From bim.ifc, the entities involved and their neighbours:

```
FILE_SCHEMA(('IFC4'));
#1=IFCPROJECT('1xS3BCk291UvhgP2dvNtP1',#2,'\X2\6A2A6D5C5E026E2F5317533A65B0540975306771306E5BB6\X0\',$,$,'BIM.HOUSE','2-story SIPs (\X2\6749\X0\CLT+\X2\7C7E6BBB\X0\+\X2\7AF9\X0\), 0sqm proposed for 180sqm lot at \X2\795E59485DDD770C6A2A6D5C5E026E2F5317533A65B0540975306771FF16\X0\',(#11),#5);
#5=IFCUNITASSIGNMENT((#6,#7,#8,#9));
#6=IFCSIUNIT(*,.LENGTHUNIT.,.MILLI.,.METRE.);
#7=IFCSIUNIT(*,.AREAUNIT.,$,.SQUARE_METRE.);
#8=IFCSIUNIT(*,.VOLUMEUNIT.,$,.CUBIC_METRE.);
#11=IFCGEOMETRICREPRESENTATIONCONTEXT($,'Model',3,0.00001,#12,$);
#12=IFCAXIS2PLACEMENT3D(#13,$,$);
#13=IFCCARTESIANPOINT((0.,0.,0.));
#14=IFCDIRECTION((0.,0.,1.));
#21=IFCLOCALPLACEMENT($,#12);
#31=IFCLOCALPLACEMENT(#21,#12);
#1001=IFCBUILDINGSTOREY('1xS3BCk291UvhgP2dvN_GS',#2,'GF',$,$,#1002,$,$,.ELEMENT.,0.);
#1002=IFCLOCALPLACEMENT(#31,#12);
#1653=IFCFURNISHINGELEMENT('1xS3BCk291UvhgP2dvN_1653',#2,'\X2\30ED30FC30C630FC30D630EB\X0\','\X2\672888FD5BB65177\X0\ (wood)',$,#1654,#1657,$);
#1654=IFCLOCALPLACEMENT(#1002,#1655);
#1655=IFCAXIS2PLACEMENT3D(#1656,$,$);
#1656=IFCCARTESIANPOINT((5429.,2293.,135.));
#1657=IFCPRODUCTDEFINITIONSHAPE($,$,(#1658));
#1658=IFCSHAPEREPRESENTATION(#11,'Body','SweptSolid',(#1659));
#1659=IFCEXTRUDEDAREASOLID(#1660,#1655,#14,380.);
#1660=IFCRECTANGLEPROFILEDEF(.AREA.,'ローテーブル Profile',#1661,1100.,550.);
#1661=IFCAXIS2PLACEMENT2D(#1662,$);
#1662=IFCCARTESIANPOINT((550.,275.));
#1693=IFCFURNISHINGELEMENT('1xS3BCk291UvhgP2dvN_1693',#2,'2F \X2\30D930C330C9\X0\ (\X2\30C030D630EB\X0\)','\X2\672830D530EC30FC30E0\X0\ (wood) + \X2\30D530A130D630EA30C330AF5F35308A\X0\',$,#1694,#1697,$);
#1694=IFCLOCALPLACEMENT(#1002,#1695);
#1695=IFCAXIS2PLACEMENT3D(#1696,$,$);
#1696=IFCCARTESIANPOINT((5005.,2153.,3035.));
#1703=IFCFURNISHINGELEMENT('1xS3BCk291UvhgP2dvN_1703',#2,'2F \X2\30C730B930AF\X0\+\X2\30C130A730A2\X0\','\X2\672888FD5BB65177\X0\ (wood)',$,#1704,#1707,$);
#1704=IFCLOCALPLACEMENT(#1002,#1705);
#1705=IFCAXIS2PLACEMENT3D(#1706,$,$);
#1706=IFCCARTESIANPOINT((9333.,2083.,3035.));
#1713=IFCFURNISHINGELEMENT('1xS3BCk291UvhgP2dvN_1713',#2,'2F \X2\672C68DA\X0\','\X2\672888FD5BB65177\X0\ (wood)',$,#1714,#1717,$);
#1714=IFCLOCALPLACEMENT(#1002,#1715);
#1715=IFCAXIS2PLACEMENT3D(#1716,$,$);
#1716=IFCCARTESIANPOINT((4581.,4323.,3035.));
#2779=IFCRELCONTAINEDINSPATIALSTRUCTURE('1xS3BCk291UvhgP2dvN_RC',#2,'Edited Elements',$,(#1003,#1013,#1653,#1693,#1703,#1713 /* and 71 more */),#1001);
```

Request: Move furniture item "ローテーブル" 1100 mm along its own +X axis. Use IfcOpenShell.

```python
import ifcopenshell
import ifcopenshell.api.geometry
import ifcopenshell.util.placement
import ifcopenshell.util.unit

model = ifcopenshell.open("bim.ifc")
unit_scale = ifcopenshell.util.unit.calculate_unit_scale(model)

item = model.by_guid("1xS3BCk291UvhgP2dvN_1653")
matrix = ifcopenshell.util.placement.get_local_placement(item.ObjectPlacement)
matrix[:3, 3] += matrix[:3, 0] * 1.1 / unit_scale
ifcopenshell.api.geometry.edit_object_placement(model, product=item, matrix=matrix, is_si=False)

print(ifcopenshell.util.placement.get_local_placement(item.ObjectPlacement).round(3) + 0.0)

model.write("bim-out.ifc")
```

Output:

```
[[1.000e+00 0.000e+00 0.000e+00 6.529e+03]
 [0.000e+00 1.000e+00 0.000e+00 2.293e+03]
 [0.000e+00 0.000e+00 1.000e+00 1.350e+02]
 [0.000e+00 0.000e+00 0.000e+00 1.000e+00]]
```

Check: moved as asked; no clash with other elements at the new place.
